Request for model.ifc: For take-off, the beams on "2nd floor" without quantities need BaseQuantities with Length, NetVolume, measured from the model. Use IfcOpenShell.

First a look at what the model holds.

```python
import ifcopenshell
import ifcopenshell.util.element
import ifcopenshell.util.unit

model = ifcopenshell.open("model.ifc")
print(model.schema)
for unit_type in ("LENGTHUNIT", "AREAUNIT", "VOLUMEUNIT"):
    print(unit_type, ifcopenshell.util.unit.calculate_unit_scale(model, unit_type))
storey = next(s for s in model.by_type("IfcBuildingStorey") if s.Name == "2nd floor")
beams = [e for e in ifcopenshell.util.element.get_decomposition(storey) if e.is_a("IfcBeam")]
for e in sorted(beams, key=lambda e: e.id()):
    print(e.id(), e.is_a(), e.Name, list(ifcopenshell.util.element.get_psets(e, qtos_only=True)), sep=" | ")
```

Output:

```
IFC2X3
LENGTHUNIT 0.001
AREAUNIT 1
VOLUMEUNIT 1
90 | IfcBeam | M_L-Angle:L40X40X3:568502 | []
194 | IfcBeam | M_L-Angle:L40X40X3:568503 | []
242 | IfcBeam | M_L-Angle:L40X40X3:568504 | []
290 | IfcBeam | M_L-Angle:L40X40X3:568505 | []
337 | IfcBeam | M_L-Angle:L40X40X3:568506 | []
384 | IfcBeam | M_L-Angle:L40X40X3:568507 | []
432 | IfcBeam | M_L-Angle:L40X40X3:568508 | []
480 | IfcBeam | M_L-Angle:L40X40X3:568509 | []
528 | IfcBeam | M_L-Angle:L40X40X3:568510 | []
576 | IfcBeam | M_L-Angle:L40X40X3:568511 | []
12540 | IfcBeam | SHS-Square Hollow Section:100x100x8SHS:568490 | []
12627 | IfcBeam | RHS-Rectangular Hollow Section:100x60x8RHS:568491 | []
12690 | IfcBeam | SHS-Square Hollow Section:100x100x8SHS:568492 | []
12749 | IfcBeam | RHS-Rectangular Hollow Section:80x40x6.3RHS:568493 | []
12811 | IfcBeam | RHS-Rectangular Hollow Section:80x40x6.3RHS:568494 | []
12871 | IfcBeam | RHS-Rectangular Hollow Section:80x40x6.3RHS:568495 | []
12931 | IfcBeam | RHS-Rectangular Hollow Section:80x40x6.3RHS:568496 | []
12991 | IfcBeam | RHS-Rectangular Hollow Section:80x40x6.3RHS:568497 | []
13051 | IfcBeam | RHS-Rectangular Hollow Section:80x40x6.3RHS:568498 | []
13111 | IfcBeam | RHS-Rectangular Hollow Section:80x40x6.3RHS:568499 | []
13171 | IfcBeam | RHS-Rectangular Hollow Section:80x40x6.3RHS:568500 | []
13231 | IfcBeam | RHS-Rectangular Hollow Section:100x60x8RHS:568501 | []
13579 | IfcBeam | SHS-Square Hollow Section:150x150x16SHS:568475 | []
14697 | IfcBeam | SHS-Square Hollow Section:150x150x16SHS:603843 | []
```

```python
import ifcopenshell
import ifcopenshell.api.pset
import ifcopenshell.geom
import ifcopenshell.util.element
import ifcopenshell.util.shape
import ifcopenshell.util.unit

model = ifcopenshell.open("model.ifc")
unit_scale = ifcopenshell.util.unit.calculate_unit_scale(model)
volume_scale = ifcopenshell.util.unit.calculate_unit_scale(model, "VOLUMEUNIT")
settings = ifcopenshell.geom.settings()

storey = next(s for s in model.by_type("IfcBuildingStorey") if s.Name == "2nd floor")
beams = [e for e in ifcopenshell.util.element.get_decomposition(storey) if e.is_a("IfcBeam")]

for e in sorted(beams, key=lambda e: e.id()):
    if ifcopenshell.util.element.get_psets(e, qtos_only=True, should_inherit=False):
        continue
    # Geometry comes back in metres, in the element's own axes.
    shape = ifcopenshell.geom.create_shape(settings, e)
    values = {
        "Length": ifcopenshell.util.shape.get_max_xyz(shape.geometry) / unit_scale,
        "NetVolume": ifcopenshell.util.shape.get_volume(shape.geometry) / volume_scale,
    }
    qto = ifcopenshell.api.pset.add_qto(model, product=e, name="BaseQuantities")
    ifcopenshell.api.pset.edit_qto(model, qto=qto, properties=values)
    print(e.id(), {k: round(v, 3) for k, v in values.items()})

model.write("model_edited.ifc")
```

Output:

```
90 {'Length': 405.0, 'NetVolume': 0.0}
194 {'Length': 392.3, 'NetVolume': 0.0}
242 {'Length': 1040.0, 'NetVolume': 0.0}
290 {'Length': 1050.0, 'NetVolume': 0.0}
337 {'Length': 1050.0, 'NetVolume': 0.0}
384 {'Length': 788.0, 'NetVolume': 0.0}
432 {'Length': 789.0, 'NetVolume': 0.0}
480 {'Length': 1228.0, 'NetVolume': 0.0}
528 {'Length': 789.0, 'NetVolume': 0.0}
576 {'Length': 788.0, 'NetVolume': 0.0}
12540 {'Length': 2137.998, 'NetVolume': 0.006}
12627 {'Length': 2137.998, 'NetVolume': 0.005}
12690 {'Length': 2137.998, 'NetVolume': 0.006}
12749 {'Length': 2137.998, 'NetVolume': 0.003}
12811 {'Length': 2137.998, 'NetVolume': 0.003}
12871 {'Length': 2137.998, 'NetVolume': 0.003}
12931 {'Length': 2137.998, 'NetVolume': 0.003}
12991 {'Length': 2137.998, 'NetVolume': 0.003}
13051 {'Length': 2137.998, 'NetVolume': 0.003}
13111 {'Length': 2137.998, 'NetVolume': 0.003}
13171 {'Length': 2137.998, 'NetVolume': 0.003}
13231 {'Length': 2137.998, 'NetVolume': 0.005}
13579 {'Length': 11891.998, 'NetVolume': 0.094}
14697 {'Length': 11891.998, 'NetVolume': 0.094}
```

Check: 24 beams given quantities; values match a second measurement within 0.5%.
